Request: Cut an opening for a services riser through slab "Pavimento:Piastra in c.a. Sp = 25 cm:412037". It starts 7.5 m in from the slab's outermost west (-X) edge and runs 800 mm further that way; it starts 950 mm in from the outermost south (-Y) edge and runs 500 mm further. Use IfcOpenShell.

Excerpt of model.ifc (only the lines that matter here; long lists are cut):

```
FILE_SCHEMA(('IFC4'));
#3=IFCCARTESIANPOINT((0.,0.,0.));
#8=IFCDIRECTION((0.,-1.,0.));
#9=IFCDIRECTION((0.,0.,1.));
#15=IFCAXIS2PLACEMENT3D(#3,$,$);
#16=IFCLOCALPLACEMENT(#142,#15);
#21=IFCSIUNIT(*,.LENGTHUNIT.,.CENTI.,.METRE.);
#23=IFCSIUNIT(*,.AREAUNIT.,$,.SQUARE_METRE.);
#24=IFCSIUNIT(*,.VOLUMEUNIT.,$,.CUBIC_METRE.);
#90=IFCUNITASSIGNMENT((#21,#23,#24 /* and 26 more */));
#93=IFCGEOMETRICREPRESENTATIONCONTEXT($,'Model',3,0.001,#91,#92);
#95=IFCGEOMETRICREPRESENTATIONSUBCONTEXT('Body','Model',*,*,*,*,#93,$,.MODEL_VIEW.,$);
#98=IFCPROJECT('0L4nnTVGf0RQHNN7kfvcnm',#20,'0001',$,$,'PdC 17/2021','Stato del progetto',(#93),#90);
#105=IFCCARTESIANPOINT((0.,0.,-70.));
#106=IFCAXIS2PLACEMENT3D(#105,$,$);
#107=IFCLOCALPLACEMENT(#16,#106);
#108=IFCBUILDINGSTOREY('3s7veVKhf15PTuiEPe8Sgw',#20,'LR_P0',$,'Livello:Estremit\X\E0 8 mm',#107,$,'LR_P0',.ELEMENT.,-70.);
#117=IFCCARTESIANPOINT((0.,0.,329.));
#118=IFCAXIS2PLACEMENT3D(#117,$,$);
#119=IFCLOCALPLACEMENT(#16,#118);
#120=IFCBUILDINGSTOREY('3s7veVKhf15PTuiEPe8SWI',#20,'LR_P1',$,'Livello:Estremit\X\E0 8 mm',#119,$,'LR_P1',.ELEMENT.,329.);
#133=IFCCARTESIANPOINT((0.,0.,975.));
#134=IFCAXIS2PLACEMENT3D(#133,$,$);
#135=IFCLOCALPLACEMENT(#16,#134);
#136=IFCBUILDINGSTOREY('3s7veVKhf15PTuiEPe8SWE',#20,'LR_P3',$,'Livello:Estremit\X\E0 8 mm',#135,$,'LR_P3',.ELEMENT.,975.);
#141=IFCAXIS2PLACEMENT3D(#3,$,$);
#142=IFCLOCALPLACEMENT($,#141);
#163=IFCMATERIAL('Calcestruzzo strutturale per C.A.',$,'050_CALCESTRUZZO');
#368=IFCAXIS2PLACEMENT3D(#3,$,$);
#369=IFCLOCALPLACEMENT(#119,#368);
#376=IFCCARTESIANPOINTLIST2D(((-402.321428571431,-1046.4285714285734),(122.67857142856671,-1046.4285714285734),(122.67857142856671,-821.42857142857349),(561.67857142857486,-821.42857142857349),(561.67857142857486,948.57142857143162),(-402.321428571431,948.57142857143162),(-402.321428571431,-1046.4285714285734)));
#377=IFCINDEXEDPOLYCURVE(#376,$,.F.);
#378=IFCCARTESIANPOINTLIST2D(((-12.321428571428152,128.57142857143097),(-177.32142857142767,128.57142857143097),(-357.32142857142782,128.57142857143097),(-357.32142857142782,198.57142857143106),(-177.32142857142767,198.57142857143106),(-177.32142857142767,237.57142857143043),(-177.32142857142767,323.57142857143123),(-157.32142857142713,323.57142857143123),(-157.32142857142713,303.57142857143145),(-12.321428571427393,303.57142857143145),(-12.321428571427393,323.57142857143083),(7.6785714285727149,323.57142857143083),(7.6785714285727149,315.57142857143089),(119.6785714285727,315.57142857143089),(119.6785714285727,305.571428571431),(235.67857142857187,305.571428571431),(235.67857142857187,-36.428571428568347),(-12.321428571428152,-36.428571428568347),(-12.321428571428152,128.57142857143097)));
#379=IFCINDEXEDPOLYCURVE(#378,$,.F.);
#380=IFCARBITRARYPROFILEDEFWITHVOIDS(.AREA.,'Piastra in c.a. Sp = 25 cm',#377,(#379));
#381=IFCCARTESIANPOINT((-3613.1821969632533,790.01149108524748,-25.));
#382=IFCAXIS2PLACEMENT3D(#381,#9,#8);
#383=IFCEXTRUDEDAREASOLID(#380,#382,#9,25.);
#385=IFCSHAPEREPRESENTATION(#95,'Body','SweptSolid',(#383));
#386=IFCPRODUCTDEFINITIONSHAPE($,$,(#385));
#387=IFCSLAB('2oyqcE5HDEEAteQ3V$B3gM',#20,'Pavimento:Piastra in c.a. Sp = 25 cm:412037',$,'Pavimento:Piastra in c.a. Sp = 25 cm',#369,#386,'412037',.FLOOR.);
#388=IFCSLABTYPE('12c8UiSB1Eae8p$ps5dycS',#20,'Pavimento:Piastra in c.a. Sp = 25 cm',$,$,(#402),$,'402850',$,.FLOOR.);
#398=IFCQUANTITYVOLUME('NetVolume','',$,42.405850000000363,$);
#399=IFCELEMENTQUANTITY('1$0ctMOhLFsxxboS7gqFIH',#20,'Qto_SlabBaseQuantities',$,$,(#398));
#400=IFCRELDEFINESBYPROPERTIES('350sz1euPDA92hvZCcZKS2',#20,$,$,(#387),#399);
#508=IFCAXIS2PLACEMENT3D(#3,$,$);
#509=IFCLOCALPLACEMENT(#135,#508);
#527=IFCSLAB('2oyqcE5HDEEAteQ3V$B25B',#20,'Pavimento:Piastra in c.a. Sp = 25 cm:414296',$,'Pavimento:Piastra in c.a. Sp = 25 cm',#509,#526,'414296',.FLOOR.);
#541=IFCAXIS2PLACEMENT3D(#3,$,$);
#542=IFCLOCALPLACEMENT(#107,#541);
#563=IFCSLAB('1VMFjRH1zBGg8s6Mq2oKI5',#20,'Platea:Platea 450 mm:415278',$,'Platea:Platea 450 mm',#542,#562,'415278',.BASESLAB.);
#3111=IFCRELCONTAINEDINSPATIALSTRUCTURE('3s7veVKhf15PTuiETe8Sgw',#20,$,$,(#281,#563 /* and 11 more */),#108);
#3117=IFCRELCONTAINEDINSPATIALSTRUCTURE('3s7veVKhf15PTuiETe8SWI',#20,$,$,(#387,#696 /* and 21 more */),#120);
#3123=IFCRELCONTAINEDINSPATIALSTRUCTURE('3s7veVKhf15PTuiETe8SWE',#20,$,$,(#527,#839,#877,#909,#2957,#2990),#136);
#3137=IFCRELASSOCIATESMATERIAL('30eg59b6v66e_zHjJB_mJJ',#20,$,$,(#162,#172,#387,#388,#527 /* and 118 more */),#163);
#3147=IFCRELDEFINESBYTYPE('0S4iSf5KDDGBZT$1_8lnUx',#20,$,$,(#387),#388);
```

```python
import numpy as np
import ifcopenshell
import ifcopenshell.api.feature
import ifcopenshell.api.geometry
import ifcopenshell.api.pset
import ifcopenshell.api.root
import ifcopenshell.geom
import ifcopenshell.util.element
import ifcopenshell.util.placement
import ifcopenshell.util.representation
import ifcopenshell.util.shape
import ifcopenshell.util.unit

model = ifcopenshell.open("model.ifc")
unit_scale = ifcopenshell.util.unit.calculate_unit_scale(model)
volume_scale = ifcopenshell.util.unit.calculate_unit_scale(model, "VOLUMEUNIT")
settings = ifcopenshell.geom.settings()


def volume(element):
    """Net volume in cubic metres, openings subtracted."""
    shape = ifcopenshell.geom.create_shape(settings, element)
    return ifcopenshell.util.shape.get_volume(shape.geometry)


slab = model.by_guid("2oyqcE5HDEEAteQ3V$B3gM")
before = volume(slab)

# Extent in the slab's own axes, in metres. The edges named are its -X and -Y sides.
slab_shape = ifcopenshell.geom.create_shape(settings, slab)
vertices = ifcopenshell.util.shape.get_vertices(slab_shape.geometry)
x_min, y_min, bottom = vertices.min(axis=0)
top = vertices[:, 2].max()

opening = ifcopenshell.api.root.create_entity(model, ifc_class="IfcOpeningElement", name="Services riser opening", predefined_type="OPENING")
context = ifcopenshell.util.representation.get_context(model, "Model", "Body", "MODEL_VIEW")
width, depth = 0.8, 0.5
outline = [(0.0, 0.0), (width, 0.0), (width, depth), (0.0, depth), (0.0, 0.0)]
# Overshoot both faces by 50 mm so the cut is clean.
shape = ifcopenshell.api.geometry.add_slab_representation(
    model, context=context, depth=top - bottom + 0.1, polyline=outline
)
ifcopenshell.api.geometry.assign_representation(model, product=opening, representation=shape)

matrix = ifcopenshell.util.placement.get_local_placement(slab.ObjectPlacement)
matrix[:, 3] = matrix @ np.append(np.array([x_min + 7.5, y_min + 0.95, bottom - 0.05]) / unit_scale, 1.0)
ifcopenshell.api.geometry.edit_object_placement(model, product=opening, matrix=matrix, is_si=False)
ifcopenshell.api.feature.add_feature(model, feature=opening, element=slab)

after = volume(slab)

# Update the slab's stored quantities.
qto = model.by_id(ifcopenshell.util.element.get_pset(slab, "Qto_SlabBaseQuantities", should_inherit=False)["id"])
ifcopenshell.api.pset.edit_qto(model, qto=qto, properties={"NetVolume": after / volume_scale})

print(f"slab volume {before:.3f} -> {after:.3f} m3")

model.write("model_updated.ifc")
```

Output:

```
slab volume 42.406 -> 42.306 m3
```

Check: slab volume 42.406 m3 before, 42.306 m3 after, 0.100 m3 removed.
